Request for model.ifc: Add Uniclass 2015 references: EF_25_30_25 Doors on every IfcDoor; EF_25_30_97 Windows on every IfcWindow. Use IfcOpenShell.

First a look at what the model holds.

```python
import ifcopenshell

model = ifcopenshell.open("model.ifc")
print(model.schema)
print("classifications:", [c.Name for c in model.by_type("IfcClassification")])
for ifc_class in ("IfcDoor", "IfcRoof", "IfcStair", "IfcWall", "IfcWindow"):
    print(ifc_class, len(model.by_type(ifc_class)))
```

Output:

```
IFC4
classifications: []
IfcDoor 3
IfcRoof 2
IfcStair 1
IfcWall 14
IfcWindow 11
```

```python
import ifcopenshell
import ifcopenshell.api.classification

model = ifcopenshell.open("model.ifc")

system = ifcopenshell.api.classification.add_classification(model, classification="Uniclass 2015")

codes = {
    "IfcDoor": ("EF_25_30_25", "Doors"),
    "IfcWindow": ("EF_25_30_97", "Windows"),
}
for ifc_class, (code, name) in codes.items():
    products = model.by_type(ifc_class)
    ifcopenshell.api.classification.add_reference(
        model, products=products, classification=system, identification=code, name=name
    )
    print(code, len(products))

model.write("model-out.ifc")
```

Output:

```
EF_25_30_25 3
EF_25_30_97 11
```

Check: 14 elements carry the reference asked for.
